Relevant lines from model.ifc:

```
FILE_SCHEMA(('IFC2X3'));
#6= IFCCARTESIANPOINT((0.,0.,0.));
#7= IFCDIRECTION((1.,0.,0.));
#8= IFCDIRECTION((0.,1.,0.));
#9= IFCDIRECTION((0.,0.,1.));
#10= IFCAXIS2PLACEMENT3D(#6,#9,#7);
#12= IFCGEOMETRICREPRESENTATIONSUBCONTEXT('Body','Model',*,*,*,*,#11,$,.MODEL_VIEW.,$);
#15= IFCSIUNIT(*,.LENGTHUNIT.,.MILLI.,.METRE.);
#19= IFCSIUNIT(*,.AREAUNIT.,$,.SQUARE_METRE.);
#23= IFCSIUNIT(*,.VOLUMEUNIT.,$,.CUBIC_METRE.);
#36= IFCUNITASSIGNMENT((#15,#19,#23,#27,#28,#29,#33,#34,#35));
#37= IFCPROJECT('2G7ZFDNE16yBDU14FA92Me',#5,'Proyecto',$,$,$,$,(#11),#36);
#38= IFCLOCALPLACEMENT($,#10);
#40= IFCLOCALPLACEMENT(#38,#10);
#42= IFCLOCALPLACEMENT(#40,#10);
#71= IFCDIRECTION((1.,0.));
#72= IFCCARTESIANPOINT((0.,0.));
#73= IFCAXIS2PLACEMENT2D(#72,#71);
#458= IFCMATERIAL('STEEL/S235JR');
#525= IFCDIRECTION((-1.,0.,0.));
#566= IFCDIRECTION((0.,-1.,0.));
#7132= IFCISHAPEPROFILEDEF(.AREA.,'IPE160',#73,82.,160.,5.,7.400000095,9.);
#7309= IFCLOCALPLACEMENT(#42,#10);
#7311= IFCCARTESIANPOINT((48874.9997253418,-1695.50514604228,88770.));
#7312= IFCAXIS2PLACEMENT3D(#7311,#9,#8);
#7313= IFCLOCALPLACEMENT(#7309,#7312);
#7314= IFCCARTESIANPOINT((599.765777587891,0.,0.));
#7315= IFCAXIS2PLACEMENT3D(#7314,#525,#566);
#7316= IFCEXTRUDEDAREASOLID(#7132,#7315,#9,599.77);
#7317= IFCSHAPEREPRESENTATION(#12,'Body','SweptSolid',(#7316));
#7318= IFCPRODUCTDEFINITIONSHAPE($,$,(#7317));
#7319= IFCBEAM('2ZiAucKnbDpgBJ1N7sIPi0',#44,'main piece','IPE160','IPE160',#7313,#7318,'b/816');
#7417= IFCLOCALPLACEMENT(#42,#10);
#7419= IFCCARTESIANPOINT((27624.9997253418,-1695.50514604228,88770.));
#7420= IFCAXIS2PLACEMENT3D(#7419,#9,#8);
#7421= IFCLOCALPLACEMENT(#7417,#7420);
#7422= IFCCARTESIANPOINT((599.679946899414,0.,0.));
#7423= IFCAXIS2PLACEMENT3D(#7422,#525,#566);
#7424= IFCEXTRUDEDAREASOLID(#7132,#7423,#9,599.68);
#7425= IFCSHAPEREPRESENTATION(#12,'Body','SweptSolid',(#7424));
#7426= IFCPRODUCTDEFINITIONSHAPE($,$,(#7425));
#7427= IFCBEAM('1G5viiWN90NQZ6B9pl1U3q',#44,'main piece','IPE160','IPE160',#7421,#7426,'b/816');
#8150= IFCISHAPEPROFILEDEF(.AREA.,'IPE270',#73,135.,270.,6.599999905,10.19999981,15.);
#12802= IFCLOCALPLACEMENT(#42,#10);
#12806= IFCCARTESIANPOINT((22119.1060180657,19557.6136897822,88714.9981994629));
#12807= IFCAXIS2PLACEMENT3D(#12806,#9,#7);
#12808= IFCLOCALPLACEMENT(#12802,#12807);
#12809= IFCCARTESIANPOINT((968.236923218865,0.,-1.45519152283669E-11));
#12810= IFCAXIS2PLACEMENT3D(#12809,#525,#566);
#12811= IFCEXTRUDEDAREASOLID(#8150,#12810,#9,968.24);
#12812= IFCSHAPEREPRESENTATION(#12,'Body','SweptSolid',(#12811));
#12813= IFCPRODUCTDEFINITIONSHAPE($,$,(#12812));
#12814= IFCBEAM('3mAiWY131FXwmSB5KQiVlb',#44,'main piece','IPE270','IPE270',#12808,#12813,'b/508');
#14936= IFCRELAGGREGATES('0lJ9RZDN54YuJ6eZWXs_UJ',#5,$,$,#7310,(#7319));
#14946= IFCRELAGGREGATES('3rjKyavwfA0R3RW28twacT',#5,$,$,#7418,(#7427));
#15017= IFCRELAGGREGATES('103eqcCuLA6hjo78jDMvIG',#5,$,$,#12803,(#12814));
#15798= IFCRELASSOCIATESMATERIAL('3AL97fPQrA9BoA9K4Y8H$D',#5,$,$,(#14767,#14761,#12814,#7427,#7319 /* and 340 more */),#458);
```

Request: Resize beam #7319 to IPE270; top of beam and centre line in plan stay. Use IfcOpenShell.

```python
import ifcopenshell
import ifcopenshell.util.element
import ifcopenshell.util.representation

model = ifcopenshell.open("model.ifc")

member = model.by_guid("2ZiAucKnbDpgBJ1N7sIPi0")
source = next(p for p in model.by_type("IfcIShapeProfileDef") if p.ProfileName == "IPE270")

body = ifcopenshell.util.representation.get_representation(member, "Model", "Body")
solid = body.Items[0]
old_profile = solid.SweptArea

# Copy the section's sizes but keep this member's own profile position.
profile = ifcopenshell.util.element.copy(model, source)
# Profiles are centred, so shift by half the change in depth to hold the top.
shift = (old_profile.OverallDepth - profile.OverallDepth) / 2
x, y = old_profile.Position.Location.Coordinates
up = (0.0, 1.0)  # upwards, in the solid's own plane
location = model.createIfcCartesianPoint((x + up[0] * shift, y + up[1] * shift))
profile.Position = model.createIfcAxis2Placement2D(location, old_profile.Position.RefDirection)
solid.SweptArea = profile
if not model.get_total_inverses(old_profile):
    ifcopenshell.util.element.remove_deep2(model, old_profile)
member.Description = member.Description.replace("IPE160", "IPE270")
member.ObjectType = member.ObjectType.replace("IPE160", "IPE270")

print(solid.SweptArea)

model.write("model-out.ifc")
```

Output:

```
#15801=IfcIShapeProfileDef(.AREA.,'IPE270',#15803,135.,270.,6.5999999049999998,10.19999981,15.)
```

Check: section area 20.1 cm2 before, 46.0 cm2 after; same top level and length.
